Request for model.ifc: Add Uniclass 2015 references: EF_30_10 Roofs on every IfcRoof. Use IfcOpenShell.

First a look at what the model holds.

```python
import ifcopenshell

model = ifcopenshell.open("model.ifc")
print(model.schema)
print("classifications:", [c.Name for c in model.by_type("IfcClassification")])
for ifc_class in ("IfcDoor", "IfcRoof", "IfcStair", "IfcWall", "IfcWindow"):
    print(ifc_class, len(model.by_type(ifc_class)))
```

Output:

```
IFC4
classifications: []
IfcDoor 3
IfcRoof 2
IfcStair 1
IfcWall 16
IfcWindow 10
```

```python
import ifcopenshell
import ifcopenshell.api.classification

model = ifcopenshell.open("model.ifc")

system = ifcopenshell.api.classification.add_classification(model, classification="Uniclass 2015")

codes = {
    "IfcRoof": ("EF_30_10", "Roofs"),
}
for ifc_class, (code, name) in codes.items():
    products = model.by_type(ifc_class)
    ifcopenshell.api.classification.add_reference(
        model, products=products, classification=system, identification=code, name=name
    )
    print(code, len(products))

model.write("model_rev.ifc")
```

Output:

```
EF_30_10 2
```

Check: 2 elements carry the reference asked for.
